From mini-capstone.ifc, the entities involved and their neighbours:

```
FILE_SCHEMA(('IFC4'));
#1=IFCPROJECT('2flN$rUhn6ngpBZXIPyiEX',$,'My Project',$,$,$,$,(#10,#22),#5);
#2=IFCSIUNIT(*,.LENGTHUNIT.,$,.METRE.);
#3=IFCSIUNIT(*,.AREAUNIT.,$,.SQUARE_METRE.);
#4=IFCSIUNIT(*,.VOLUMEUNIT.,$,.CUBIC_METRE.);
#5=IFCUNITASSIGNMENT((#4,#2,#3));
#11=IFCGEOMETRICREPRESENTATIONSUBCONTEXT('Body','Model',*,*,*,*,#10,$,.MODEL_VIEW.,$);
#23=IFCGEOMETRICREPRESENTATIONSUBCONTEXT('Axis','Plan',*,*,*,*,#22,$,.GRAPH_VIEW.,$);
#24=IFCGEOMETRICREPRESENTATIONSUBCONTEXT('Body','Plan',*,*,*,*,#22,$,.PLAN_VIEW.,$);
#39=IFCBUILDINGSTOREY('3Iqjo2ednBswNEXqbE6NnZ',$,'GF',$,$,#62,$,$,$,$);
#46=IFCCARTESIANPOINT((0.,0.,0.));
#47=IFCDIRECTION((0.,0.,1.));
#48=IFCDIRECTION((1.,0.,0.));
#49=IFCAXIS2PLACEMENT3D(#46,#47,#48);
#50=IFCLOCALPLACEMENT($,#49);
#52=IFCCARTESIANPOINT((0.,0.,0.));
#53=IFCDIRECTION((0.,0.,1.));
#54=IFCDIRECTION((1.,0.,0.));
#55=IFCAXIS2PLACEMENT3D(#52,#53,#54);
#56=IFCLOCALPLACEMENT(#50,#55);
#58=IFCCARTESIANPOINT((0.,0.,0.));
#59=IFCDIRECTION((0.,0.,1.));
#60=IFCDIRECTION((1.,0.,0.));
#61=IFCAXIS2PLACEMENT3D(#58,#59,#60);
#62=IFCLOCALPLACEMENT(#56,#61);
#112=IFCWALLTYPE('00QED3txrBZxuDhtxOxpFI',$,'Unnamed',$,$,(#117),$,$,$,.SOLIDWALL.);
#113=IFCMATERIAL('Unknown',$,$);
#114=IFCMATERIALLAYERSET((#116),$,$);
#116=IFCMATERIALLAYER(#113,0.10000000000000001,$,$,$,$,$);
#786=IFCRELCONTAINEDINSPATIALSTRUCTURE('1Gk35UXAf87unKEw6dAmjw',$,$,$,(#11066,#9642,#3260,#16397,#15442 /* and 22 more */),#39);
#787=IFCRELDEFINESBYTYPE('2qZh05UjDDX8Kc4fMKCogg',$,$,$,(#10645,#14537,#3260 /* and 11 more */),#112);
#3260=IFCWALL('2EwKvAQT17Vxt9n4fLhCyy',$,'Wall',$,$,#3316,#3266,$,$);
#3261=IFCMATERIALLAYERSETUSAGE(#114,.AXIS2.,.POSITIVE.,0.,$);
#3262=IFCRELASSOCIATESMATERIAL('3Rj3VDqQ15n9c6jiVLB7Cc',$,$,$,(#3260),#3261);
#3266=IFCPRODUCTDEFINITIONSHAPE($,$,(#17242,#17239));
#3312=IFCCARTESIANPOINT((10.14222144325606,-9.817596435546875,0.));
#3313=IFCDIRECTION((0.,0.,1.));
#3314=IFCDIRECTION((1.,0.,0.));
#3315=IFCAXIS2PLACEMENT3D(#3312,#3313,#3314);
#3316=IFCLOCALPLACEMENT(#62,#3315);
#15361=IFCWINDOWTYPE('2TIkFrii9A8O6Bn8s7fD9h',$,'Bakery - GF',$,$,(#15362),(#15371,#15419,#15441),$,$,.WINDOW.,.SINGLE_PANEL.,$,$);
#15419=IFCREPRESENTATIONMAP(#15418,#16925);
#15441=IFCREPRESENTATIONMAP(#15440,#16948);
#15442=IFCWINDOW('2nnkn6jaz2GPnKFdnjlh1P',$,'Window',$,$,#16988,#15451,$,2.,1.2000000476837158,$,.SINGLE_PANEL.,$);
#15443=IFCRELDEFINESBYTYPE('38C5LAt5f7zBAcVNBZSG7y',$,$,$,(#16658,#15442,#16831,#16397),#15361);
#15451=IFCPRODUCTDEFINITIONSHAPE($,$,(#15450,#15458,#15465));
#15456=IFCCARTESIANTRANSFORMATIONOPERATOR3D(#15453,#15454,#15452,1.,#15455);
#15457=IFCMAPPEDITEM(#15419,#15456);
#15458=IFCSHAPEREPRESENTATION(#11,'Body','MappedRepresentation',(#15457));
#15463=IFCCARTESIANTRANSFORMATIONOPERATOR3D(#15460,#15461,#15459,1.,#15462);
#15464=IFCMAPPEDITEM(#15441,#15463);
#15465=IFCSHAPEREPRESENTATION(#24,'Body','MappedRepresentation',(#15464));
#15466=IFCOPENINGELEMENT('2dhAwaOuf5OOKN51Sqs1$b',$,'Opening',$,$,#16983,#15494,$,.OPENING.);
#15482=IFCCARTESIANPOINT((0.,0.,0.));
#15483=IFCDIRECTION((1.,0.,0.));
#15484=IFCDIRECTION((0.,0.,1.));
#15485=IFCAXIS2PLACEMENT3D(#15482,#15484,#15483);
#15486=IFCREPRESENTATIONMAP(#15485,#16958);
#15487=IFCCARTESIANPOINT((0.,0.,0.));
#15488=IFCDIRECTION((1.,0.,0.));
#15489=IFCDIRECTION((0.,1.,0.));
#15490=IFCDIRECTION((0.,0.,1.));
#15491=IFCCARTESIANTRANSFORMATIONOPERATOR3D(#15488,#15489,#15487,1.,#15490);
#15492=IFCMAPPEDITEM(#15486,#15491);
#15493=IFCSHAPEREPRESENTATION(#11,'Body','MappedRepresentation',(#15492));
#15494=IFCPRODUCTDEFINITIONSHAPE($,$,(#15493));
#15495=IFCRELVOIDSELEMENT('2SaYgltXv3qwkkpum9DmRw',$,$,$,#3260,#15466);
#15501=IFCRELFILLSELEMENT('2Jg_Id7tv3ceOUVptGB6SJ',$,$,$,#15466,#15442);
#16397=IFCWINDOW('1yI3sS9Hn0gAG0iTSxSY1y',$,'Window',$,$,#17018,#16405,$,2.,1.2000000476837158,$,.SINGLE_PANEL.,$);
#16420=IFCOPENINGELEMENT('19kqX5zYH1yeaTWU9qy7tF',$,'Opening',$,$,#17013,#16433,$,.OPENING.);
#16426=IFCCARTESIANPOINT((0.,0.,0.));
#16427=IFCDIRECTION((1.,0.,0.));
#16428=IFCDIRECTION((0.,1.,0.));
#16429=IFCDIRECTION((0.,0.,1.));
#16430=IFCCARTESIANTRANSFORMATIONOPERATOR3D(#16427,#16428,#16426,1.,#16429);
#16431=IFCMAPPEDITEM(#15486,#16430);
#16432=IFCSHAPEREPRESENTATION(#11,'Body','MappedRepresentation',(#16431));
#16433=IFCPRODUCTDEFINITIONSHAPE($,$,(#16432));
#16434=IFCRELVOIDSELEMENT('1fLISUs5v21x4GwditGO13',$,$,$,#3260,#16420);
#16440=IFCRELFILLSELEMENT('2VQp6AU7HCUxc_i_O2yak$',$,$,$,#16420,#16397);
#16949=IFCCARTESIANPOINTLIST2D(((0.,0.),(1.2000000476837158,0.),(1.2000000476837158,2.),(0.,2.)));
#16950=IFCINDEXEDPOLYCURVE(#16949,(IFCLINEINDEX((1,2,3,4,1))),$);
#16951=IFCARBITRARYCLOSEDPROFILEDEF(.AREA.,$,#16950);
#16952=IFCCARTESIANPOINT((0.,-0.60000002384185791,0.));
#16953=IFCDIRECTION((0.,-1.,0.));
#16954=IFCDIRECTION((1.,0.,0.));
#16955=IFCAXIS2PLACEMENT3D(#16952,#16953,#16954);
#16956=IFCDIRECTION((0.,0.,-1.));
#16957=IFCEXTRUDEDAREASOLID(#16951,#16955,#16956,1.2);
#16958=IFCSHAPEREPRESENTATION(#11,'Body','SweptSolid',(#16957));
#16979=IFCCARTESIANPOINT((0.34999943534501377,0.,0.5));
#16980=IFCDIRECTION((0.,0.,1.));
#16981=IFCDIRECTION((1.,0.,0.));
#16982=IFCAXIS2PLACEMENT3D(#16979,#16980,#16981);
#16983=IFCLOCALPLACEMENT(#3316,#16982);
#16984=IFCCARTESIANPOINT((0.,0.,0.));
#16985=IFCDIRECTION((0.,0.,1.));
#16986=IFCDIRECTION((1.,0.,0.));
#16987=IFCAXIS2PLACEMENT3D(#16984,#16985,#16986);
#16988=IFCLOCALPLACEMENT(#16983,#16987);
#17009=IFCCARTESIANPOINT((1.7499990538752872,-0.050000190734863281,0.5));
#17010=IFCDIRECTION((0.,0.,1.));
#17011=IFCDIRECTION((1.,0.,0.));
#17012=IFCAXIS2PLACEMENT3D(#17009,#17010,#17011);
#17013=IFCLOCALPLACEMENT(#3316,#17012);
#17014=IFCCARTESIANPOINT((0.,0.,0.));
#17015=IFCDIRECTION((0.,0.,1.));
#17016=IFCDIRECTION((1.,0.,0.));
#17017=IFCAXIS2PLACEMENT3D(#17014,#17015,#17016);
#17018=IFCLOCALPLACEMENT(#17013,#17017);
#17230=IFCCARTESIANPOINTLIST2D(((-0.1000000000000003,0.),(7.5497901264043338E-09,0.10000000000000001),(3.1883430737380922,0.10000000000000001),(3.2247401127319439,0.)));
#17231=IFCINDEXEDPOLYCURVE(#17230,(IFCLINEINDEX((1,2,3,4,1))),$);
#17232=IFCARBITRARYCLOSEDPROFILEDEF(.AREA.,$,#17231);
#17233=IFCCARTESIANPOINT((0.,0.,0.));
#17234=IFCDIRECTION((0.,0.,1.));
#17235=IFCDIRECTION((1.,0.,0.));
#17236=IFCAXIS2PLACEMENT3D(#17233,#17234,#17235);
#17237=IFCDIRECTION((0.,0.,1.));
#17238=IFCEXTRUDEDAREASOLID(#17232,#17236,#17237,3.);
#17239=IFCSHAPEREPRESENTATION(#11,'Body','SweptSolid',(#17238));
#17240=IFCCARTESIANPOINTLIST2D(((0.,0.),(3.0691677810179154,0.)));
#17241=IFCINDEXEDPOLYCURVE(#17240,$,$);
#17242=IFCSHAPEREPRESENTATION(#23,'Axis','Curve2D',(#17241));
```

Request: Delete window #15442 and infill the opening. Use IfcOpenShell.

```python
import ifcopenshell
import ifcopenshell.api.feature
import ifcopenshell.api.root
import ifcopenshell.geom
import ifcopenshell.util.shape

model = ifcopenshell.open("mini-capstone.ifc")
settings = ifcopenshell.geom.settings()


def volume(element):
    """Net volume in cubic metres, openings subtracted."""
    shape = ifcopenshell.geom.create_shape(settings, element)
    return ifcopenshell.util.shape.get_volume(shape.geometry)


window = model.by_guid("2nnkn6jaz2GPnKFdnjlh1P")
opening = window.FillsVoids[0].RelatingOpeningElement
wall = opening.VoidsElements[0].RelatingBuildingElement
before = volume(wall)

ifcopenshell.api.root.remove_product(model, product=window)
ifcopenshell.api.feature.remove_feature(model, feature=opening)

after = volume(wall)

print(f"wall volume {before:.3f} -> {after:.3f} m3")

model.write("mini-capstone_v2.ifc")
```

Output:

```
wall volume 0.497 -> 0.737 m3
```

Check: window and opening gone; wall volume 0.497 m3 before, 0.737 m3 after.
